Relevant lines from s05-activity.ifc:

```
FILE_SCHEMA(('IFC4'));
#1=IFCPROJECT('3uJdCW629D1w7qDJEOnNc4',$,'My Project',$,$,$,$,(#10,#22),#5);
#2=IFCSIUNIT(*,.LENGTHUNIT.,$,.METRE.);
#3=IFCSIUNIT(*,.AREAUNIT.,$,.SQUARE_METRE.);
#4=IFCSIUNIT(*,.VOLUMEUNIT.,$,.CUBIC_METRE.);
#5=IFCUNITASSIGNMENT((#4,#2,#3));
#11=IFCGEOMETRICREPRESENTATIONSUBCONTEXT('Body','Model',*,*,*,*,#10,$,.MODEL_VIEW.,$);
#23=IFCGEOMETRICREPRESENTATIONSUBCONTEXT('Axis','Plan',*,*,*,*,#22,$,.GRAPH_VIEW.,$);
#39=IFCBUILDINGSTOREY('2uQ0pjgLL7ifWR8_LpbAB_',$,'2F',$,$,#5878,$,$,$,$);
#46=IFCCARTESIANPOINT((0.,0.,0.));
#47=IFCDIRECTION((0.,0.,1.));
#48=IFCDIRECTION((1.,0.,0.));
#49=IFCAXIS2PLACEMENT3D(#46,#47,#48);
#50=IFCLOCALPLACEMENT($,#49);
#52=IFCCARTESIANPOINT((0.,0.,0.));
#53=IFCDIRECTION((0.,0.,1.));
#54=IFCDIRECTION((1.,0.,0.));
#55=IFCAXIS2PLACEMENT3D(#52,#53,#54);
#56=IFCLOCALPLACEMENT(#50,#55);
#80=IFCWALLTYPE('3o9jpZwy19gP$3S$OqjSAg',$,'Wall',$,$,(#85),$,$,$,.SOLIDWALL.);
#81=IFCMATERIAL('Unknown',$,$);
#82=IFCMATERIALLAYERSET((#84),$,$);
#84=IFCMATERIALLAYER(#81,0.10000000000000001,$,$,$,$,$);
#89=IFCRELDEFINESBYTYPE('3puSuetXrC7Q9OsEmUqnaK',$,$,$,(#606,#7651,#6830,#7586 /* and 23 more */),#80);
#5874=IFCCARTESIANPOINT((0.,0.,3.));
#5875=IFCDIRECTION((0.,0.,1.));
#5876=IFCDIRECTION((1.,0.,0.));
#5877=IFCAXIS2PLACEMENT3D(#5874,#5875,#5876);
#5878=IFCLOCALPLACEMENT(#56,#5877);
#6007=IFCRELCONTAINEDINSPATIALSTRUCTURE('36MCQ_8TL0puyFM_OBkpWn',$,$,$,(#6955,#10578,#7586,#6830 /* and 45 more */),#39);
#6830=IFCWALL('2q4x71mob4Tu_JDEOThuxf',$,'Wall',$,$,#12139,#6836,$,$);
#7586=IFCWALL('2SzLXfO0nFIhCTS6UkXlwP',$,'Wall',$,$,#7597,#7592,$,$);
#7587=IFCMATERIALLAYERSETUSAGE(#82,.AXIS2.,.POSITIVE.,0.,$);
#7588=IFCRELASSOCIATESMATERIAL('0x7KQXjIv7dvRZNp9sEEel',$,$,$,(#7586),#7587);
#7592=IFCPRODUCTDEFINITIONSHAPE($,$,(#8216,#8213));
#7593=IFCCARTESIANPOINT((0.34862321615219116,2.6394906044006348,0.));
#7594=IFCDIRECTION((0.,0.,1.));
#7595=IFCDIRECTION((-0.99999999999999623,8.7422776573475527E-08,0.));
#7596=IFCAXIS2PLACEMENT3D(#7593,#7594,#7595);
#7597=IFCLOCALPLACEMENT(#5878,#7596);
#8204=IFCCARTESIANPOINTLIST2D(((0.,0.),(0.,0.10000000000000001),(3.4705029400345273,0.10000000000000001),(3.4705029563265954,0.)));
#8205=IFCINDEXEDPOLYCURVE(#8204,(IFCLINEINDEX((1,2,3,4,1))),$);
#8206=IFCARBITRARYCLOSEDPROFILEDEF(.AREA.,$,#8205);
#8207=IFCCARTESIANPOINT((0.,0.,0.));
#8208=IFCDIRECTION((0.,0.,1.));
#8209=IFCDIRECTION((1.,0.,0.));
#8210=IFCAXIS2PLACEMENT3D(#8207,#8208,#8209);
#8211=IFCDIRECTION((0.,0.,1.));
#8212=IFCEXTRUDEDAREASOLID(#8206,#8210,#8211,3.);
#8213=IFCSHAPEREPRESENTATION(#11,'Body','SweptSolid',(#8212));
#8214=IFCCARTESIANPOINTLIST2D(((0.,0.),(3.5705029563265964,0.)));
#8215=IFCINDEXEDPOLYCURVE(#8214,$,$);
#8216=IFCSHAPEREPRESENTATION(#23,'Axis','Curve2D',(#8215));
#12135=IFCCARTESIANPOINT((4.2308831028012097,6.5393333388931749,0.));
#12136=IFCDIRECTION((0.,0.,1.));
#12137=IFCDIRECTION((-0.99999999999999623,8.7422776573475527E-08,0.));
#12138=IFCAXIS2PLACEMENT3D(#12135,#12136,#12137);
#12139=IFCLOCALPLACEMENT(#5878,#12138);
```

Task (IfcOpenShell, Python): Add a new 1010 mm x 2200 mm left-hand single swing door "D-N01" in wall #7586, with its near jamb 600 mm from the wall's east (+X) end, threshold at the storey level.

```python
import numpy as np
import ifcopenshell
import ifcopenshell.api.feature
import ifcopenshell.api.geometry
import ifcopenshell.api.root
import ifcopenshell.api.spatial
import ifcopenshell.geom
import ifcopenshell.util.element
import ifcopenshell.util.placement
import ifcopenshell.util.representation
import ifcopenshell.util.shape
import ifcopenshell.util.unit

model = ifcopenshell.open("s05-activity.ifc")
unit_scale = ifcopenshell.util.unit.calculate_unit_scale(model)
settings = ifcopenshell.geom.settings()


def volume(element):
    """Net volume in cubic metres, openings subtracted."""
    shape = ifcopenshell.geom.create_shape(settings, element)
    return ifcopenshell.util.shape.get_volume(shape.geometry)


wall = model.by_guid("2SzLXfO0nFIhCTS6UkXlwP")
storey = ifcopenshell.util.element.get_container(wall, ifc_class="IfcBuildingStorey")
context = ifcopenshell.util.representation.get_context(model, "Model", "Body", "MODEL_VIEW")
before = volume(wall)

width, height, from_end, sill = 1.01, 2.2, 0.6, 0.0  # metres

# The wall runs along its own X axis, and the end named is its -X end.
wall_shape = ifcopenshell.geom.create_shape(settings, wall)
x, y, z = ifcopenshell.util.shape.get_vertices(wall_shape.geometry).T
start = x.min() + from_end
face, thickness = float(y.min()), float(y.max() - y.min())
wall_matrix = ifcopenshell.util.placement.get_local_placement(wall.ObjectPlacement)
level = ifcopenshell.util.placement.get_local_placement(storey.ObjectPlacement)[2, 3]


def in_wall(x, y):
    """Placement at x, y metres in the wall's axes, at sill height."""
    matrix = wall_matrix.copy()
    matrix[:, 3] = wall_matrix @ np.array([x / unit_scale, y / unit_scale, 0.0, 1.0])
    matrix[2, 3] = level + sill / unit_scale
    return matrix


# Opening: a box that overshoots both wall faces by 50 mm.
opening = ifcopenshell.api.root.create_entity(model, ifc_class="IfcOpeningElement", predefined_type="OPENING")
box = ifcopenshell.api.geometry.add_wall_representation(
    model, context=context, length=width, height=height, thickness=thickness + 0.1
)
ifcopenshell.api.geometry.assign_representation(model, product=opening, representation=box)
ifcopenshell.api.geometry.edit_object_placement(model, product=opening, matrix=in_wall(start, face - 0.05), is_si=False)
ifcopenshell.api.feature.add_feature(model, feature=opening, element=wall)

door = ifcopenshell.api.root.create_entity(model, ifc_class="IfcDoor", name="D-N01", predefined_type="DOOR")
door.OverallWidth, door.OverallHeight = width / unit_scale, height / unit_scale
door.OperationType = "SINGLE_SWING_LEFT"
body = ifcopenshell.api.geometry.add_door_representation(
    model,
    context=context,
    overall_width=door.OverallWidth,
    overall_height=door.OverallHeight,
    operation_type="SINGLE_SWING_LEFT",
    lining_properties={"LiningDepth": thickness / unit_scale, "ThresholdDepth": thickness / unit_scale},
)
ifcopenshell.api.geometry.assign_representation(model, product=door, representation=body)
ifcopenshell.api.spatial.assign_container(model, products=[door], relating_structure=storey)
ifcopenshell.api.feature.add_filling(model, opening=opening, element=door)

# The lining spans the wall, so the door starts at the wall face.
ifcopenshell.api.geometry.edit_object_placement(model, product=door, matrix=in_wall(start, face), is_si=False)

after = volume(wall)

print(f"wall volume {before:.3f} -> {after:.3f} m3")

model.write("s05-activity_rev.ifc")
```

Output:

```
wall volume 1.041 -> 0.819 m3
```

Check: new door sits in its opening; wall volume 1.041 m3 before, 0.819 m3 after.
